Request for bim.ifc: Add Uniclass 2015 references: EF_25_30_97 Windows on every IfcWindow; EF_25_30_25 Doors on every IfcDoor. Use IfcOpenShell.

First a look at what the model holds.

```python
import ifcopenshell

model = ifcopenshell.open("bim.ifc")
print(model.schema)
print("classifications:", [c.Name for c in model.by_type("IfcClassification")])
for ifc_class in ("IfcDoor", "IfcRoof", "IfcStair", "IfcWall", "IfcWindow"):
    print(ifc_class, len(model.by_type(ifc_class)))
```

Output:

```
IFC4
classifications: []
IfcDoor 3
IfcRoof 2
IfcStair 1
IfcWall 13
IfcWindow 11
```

```python
import ifcopenshell
import ifcopenshell.api.classification

model = ifcopenshell.open("bim.ifc")

system = ifcopenshell.api.classification.add_classification(model, classification="Uniclass 2015")

codes = {
    "IfcWindow": ("EF_25_30_97", "Windows"),
    "IfcDoor": ("EF_25_30_25", "Doors"),
}
for ifc_class, (code, name) in codes.items():
    products = model.by_type(ifc_class)
    ifcopenshell.api.classification.add_reference(
        model, products=products, classification=system, identification=code, name=name
    )
    print(code, len(products))

model.write("bim_rev.ifc")
```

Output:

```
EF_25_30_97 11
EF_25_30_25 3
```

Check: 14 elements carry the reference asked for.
